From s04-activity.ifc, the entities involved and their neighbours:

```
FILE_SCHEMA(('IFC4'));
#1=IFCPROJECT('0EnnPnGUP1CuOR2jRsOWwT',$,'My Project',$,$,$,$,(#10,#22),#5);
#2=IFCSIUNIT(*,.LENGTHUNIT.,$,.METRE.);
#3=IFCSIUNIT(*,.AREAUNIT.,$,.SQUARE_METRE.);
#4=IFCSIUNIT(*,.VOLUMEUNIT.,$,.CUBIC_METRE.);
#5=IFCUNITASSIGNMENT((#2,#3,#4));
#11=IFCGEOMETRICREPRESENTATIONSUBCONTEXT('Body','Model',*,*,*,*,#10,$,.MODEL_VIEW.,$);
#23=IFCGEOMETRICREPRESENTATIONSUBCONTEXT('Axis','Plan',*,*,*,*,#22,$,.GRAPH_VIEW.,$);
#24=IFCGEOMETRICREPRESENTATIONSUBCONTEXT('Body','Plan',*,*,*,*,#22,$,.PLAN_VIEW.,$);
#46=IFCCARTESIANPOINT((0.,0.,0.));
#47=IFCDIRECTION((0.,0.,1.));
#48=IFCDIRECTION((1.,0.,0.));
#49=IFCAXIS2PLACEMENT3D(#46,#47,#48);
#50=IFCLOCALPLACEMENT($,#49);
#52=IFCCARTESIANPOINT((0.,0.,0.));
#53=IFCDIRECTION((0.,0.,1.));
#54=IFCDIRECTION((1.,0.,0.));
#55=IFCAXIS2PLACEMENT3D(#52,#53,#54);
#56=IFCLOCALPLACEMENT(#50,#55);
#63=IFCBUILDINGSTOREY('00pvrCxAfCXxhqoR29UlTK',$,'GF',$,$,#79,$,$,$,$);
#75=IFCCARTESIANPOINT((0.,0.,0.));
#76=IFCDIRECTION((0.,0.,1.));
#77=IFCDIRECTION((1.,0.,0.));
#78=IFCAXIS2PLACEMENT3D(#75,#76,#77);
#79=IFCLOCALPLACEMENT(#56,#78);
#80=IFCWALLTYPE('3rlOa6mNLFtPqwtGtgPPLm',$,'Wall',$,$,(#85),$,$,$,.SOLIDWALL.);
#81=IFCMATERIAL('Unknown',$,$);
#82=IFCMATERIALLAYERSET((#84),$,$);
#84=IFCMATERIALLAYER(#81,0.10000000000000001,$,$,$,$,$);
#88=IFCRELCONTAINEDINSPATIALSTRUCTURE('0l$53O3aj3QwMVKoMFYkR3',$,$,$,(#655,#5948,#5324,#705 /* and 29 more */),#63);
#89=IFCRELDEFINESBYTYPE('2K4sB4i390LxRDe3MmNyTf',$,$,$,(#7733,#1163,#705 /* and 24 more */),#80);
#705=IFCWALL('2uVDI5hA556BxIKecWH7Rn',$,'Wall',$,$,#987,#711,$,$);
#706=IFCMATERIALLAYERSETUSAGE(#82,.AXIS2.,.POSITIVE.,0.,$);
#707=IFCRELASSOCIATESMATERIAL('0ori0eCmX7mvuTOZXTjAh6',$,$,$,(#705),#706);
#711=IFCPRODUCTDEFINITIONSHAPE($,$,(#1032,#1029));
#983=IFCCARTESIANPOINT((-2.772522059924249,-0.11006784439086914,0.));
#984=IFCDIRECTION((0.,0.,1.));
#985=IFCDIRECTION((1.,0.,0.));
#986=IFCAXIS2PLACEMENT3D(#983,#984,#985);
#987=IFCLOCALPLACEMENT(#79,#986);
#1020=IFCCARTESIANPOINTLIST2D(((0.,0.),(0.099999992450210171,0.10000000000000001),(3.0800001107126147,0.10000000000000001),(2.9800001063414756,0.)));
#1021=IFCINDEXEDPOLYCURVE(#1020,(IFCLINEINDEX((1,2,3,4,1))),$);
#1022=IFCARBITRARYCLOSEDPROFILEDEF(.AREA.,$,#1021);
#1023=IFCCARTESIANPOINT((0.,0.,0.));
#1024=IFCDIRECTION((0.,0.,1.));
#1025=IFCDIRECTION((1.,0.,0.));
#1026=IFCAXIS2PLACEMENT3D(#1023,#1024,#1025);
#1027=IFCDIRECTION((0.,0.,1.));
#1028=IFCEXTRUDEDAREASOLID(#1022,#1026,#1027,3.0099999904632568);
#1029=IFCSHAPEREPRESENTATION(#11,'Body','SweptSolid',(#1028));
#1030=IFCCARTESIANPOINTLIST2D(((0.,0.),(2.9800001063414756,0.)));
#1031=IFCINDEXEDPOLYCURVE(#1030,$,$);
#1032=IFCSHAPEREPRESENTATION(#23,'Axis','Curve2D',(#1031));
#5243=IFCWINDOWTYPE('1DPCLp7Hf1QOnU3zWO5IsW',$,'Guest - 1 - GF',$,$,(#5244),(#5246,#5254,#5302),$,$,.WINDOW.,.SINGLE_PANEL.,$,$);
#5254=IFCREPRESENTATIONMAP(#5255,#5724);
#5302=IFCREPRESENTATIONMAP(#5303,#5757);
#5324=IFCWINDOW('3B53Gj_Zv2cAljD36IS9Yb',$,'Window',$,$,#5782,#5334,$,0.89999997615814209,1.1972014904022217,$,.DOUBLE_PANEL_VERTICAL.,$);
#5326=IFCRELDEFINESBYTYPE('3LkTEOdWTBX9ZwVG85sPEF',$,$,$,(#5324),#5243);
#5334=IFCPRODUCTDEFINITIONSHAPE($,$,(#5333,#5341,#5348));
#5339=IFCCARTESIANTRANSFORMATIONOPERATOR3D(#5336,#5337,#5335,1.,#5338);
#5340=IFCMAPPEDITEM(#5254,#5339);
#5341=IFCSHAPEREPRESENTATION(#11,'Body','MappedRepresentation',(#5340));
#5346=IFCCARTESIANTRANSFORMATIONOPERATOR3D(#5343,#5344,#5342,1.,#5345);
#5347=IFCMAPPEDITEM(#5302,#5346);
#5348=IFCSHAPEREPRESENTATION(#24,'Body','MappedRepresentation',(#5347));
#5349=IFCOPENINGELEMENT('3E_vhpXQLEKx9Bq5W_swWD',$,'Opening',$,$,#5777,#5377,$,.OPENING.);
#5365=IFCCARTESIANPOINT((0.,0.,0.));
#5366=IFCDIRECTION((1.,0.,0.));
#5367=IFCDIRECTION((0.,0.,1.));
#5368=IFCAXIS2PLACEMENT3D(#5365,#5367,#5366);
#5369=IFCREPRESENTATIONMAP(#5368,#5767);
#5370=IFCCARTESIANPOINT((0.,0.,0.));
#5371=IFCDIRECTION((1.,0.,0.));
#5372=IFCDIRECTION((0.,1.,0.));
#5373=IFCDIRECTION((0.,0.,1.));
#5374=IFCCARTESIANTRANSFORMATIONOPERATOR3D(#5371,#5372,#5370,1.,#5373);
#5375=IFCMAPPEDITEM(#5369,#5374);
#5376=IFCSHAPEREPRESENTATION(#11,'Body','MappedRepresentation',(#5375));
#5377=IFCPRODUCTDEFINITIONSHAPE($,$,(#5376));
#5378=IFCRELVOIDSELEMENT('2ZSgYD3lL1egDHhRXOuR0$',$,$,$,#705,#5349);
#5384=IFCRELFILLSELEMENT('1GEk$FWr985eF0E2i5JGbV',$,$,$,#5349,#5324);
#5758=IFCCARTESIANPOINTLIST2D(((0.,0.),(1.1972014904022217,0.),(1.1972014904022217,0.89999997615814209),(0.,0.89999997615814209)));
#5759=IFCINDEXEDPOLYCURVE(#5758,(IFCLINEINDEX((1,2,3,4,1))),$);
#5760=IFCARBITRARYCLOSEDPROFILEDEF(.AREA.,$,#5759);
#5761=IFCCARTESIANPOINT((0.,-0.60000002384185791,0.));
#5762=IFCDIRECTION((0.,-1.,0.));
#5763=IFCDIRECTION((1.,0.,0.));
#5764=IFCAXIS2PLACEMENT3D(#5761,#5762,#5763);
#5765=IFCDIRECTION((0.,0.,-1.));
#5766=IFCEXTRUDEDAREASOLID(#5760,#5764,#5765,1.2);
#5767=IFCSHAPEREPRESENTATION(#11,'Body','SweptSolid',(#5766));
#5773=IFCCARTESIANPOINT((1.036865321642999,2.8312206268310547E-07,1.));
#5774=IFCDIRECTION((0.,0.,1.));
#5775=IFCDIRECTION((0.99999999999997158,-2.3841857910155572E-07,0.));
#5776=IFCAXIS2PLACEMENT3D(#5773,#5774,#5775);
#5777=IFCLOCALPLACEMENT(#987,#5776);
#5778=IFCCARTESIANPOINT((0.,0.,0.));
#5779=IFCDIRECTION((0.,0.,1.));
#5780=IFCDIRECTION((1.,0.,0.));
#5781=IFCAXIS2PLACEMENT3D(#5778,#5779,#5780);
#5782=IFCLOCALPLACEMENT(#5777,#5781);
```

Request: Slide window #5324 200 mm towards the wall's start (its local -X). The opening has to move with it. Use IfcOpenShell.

```python
import ifcopenshell
import ifcopenshell.api.geometry
import ifcopenshell.util.placement

model = ifcopenshell.open("s04-activity.ifc")

window = model.by_id(5324)
opening = window.FillsVoids[0].RelatingOpeningElement
wall = opening.VoidsElements[0].RelatingBuildingElement

wall_matrix = ifcopenshell.util.placement.get_local_placement(wall.ObjectPlacement)
shift = wall_matrix[:3, 0] * -0.2
before = ifcopenshell.util.placement.get_local_placement(window.ObjectPlacement)[:3, 3].copy()

# The window is placed relative to its opening, so it follows when the opening moves.
matrix = ifcopenshell.util.placement.get_local_placement(opening.ObjectPlacement)
matrix[:3, 3] += shift
ifcopenshell.api.geometry.edit_object_placement(
    model, product=opening, matrix=matrix, is_si=False, should_transform_children=True
)

after = ifcopenshell.util.placement.get_local_placement(window.ObjectPlacement)[:3, 3]
print("window moved by", (after - before).round(3) + 0.0)

model.write("s04-activity-out.ifc")
```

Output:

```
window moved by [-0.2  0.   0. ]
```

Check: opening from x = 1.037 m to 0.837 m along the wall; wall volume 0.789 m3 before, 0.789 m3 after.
